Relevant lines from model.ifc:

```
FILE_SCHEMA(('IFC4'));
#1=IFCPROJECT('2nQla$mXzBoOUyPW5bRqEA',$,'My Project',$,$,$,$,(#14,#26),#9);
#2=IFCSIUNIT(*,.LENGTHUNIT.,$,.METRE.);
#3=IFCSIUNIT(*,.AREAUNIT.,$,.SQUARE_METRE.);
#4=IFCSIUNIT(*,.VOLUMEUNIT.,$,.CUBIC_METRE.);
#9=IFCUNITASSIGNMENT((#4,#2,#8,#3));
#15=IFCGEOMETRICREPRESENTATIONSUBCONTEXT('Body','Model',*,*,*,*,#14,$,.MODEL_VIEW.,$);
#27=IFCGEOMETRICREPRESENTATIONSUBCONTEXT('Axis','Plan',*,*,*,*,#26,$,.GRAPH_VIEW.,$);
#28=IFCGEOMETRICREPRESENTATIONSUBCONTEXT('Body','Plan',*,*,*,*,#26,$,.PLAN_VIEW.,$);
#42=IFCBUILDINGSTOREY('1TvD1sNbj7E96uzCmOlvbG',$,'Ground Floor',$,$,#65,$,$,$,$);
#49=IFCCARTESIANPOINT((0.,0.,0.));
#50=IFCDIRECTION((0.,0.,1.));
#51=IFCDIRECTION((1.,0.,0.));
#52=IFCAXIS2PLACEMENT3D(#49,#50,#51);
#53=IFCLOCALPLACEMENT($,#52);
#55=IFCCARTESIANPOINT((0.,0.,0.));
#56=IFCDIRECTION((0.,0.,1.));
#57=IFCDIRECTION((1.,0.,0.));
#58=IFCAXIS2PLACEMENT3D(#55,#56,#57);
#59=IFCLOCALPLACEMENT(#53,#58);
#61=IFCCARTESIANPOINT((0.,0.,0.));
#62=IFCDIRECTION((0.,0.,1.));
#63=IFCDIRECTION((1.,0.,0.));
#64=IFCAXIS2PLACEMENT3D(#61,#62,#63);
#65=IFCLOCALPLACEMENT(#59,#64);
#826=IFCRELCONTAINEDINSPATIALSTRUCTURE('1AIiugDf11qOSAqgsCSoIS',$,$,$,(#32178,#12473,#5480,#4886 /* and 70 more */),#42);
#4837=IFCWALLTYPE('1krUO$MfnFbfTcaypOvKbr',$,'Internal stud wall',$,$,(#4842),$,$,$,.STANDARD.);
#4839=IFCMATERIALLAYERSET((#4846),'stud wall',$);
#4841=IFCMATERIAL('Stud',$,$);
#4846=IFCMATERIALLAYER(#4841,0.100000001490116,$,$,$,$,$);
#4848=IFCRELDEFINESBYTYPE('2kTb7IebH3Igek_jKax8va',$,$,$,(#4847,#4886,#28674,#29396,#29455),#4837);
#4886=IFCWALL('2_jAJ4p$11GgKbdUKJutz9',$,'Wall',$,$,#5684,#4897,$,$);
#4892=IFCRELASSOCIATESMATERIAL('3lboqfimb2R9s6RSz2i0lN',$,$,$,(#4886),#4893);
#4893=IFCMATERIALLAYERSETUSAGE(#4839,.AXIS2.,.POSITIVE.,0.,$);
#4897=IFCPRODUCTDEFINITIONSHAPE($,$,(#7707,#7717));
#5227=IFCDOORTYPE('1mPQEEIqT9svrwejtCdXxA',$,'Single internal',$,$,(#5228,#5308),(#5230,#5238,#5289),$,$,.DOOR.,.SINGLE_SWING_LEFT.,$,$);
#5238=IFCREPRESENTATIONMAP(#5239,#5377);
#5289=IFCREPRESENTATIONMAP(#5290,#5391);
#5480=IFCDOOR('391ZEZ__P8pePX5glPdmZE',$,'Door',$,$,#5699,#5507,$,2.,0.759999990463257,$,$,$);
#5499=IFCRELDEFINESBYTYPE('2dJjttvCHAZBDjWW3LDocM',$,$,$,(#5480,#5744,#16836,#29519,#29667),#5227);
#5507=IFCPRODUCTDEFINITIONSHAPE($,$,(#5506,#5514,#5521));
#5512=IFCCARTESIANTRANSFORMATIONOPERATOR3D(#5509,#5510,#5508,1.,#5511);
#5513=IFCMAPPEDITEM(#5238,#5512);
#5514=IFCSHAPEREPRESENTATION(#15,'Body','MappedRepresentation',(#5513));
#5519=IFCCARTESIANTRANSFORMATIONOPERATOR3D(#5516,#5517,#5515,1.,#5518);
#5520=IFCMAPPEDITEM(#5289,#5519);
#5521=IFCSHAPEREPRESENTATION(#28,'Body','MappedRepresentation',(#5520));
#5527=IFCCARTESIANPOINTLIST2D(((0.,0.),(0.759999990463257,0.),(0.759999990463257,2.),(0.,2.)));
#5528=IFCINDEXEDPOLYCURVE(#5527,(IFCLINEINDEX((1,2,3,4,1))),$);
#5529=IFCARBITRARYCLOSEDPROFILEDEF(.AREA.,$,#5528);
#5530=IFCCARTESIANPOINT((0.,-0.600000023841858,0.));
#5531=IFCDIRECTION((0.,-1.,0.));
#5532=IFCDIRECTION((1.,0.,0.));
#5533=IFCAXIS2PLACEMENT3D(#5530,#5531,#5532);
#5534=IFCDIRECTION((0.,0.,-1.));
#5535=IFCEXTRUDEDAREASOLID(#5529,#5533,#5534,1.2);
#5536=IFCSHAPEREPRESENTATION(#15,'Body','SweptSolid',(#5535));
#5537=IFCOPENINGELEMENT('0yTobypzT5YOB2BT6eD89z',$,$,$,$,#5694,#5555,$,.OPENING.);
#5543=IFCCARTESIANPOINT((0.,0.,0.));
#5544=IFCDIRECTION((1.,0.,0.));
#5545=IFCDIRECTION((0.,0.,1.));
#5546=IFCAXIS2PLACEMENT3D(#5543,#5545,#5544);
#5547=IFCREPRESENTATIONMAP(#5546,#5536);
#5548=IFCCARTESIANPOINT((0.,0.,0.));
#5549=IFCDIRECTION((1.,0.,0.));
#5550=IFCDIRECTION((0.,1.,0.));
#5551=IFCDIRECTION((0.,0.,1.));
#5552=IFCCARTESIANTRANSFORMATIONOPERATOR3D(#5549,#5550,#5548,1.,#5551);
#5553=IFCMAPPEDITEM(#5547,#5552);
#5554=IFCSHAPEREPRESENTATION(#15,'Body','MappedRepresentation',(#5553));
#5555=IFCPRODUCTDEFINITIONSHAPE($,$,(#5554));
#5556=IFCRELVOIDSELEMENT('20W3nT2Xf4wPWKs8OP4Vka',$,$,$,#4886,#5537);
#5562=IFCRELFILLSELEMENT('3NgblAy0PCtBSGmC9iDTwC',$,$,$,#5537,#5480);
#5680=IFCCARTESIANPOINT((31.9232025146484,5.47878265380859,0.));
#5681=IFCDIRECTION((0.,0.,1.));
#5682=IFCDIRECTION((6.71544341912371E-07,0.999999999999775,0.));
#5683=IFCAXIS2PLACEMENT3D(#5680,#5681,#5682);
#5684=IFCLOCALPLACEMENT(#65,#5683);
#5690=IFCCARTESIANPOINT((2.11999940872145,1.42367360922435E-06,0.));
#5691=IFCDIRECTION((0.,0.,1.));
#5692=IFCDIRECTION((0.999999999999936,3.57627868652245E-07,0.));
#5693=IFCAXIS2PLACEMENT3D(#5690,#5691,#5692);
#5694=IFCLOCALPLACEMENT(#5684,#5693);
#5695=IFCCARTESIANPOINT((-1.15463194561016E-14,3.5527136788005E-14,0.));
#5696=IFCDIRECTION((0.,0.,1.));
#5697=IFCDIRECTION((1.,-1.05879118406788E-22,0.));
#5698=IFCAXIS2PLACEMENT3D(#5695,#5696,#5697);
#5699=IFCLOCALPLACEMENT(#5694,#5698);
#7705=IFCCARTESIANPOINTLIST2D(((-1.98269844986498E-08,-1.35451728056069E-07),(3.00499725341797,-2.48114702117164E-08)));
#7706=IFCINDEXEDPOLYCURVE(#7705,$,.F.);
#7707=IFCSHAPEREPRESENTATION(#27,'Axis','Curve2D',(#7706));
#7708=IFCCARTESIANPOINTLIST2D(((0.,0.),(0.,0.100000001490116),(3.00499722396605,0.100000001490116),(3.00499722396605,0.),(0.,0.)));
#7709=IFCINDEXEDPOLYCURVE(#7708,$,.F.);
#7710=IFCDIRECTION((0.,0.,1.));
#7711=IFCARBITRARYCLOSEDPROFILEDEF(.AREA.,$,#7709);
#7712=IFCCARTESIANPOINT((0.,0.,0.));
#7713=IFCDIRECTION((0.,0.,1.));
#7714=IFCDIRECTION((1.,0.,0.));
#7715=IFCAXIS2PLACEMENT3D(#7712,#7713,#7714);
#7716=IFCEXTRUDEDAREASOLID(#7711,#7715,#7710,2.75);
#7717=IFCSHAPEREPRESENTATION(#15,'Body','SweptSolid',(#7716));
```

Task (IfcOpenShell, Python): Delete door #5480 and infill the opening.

```python
import ifcopenshell
import ifcopenshell.api.feature
import ifcopenshell.api.root
import ifcopenshell.geom
import ifcopenshell.util.shape

model = ifcopenshell.open("model.ifc")
settings = ifcopenshell.geom.settings()


def volume(element):
    """Net volume in cubic metres, openings subtracted."""
    shape = ifcopenshell.geom.create_shape(settings, element)
    return ifcopenshell.util.shape.get_volume(shape.geometry)


door = model.by_guid("391ZEZ__P8pePX5glPdmZE")
opening = door.FillsVoids[0].RelatingOpeningElement
wall = opening.VoidsElements[0].RelatingBuildingElement
before = volume(wall)

ifcopenshell.api.root.remove_product(model, product=door)
ifcopenshell.api.feature.remove_feature(model, feature=opening)

after = volume(wall)

print(f"wall volume {before:.3f} -> {after:.3f} m3")

model.write("model_rev.ifc")
```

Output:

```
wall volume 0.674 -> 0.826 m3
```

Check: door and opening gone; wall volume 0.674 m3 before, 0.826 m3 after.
